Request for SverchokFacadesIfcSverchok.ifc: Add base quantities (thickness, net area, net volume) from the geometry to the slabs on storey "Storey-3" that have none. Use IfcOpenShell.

First a look at what the model holds.

```python
import ifcopenshell
import ifcopenshell.util.element
import ifcopenshell.util.unit

model = ifcopenshell.open("SverchokFacadesIfcSverchok.ifc")
print(model.schema)
for unit_type in ("LENGTHUNIT", "AREAUNIT", "VOLUMEUNIT"):
    print(unit_type, ifcopenshell.util.unit.calculate_unit_scale(model, unit_type))
storey = next(s for s in model.by_type("IfcBuildingStorey") if s.Name == "Storey-3")
slabs = [e for e in ifcopenshell.util.element.get_decomposition(storey) if e.is_a("IfcSlab")]
for e in sorted(slabs, key=lambda e: e.id()):
    print(e.id(), e.is_a(), e.Name, list(ifcopenshell.util.element.get_psets(e, qtos_only=True)), sep=" | ")
```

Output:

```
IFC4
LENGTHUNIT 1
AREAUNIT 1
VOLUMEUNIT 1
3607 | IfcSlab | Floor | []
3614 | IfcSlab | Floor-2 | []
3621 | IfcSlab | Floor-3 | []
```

```python
import ifcopenshell
import ifcopenshell.api.pset
import ifcopenshell.geom
import ifcopenshell.util.element
import ifcopenshell.util.shape
import ifcopenshell.util.unit

model = ifcopenshell.open("SverchokFacadesIfcSverchok.ifc")
unit_scale = ifcopenshell.util.unit.calculate_unit_scale(model)
area_scale = ifcopenshell.util.unit.calculate_unit_scale(model, "AREAUNIT")
volume_scale = ifcopenshell.util.unit.calculate_unit_scale(model, "VOLUMEUNIT")
settings = ifcopenshell.geom.settings()

storey = next(s for s in model.by_type("IfcBuildingStorey") if s.Name == "Storey-3")
slabs = [e for e in ifcopenshell.util.element.get_decomposition(storey) if e.is_a("IfcSlab")]

for e in sorted(slabs, key=lambda e: e.id()):
    if ifcopenshell.util.element.get_psets(e, qtos_only=True, should_inherit=False):
        continue
    # Geometry comes back in metres, in the element's own axes.
    shape = ifcopenshell.geom.create_shape(settings, e)
    values = {
        "Width": ifcopenshell.util.shape.get_z(shape.geometry) / unit_scale,
        "NetArea": ifcopenshell.util.shape.get_footprint_area(shape.geometry) / area_scale,
        "NetVolume": ifcopenshell.util.shape.get_volume(shape.geometry) / volume_scale,
    }
    qto = ifcopenshell.api.pset.add_qto(model, product=e, name="Qto_SlabBaseQuantities")
    ifcopenshell.api.pset.edit_qto(model, qto=qto, properties=values)
    print(e.id(), {k: round(v, 3) for k, v in values.items()})

model.write("SverchokFacadesIfcSverchok_rev.ifc")
```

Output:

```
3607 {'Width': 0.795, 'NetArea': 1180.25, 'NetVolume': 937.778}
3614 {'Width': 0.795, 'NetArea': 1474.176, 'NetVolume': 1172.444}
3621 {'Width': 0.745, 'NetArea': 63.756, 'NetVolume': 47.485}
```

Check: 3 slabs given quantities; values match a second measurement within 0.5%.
